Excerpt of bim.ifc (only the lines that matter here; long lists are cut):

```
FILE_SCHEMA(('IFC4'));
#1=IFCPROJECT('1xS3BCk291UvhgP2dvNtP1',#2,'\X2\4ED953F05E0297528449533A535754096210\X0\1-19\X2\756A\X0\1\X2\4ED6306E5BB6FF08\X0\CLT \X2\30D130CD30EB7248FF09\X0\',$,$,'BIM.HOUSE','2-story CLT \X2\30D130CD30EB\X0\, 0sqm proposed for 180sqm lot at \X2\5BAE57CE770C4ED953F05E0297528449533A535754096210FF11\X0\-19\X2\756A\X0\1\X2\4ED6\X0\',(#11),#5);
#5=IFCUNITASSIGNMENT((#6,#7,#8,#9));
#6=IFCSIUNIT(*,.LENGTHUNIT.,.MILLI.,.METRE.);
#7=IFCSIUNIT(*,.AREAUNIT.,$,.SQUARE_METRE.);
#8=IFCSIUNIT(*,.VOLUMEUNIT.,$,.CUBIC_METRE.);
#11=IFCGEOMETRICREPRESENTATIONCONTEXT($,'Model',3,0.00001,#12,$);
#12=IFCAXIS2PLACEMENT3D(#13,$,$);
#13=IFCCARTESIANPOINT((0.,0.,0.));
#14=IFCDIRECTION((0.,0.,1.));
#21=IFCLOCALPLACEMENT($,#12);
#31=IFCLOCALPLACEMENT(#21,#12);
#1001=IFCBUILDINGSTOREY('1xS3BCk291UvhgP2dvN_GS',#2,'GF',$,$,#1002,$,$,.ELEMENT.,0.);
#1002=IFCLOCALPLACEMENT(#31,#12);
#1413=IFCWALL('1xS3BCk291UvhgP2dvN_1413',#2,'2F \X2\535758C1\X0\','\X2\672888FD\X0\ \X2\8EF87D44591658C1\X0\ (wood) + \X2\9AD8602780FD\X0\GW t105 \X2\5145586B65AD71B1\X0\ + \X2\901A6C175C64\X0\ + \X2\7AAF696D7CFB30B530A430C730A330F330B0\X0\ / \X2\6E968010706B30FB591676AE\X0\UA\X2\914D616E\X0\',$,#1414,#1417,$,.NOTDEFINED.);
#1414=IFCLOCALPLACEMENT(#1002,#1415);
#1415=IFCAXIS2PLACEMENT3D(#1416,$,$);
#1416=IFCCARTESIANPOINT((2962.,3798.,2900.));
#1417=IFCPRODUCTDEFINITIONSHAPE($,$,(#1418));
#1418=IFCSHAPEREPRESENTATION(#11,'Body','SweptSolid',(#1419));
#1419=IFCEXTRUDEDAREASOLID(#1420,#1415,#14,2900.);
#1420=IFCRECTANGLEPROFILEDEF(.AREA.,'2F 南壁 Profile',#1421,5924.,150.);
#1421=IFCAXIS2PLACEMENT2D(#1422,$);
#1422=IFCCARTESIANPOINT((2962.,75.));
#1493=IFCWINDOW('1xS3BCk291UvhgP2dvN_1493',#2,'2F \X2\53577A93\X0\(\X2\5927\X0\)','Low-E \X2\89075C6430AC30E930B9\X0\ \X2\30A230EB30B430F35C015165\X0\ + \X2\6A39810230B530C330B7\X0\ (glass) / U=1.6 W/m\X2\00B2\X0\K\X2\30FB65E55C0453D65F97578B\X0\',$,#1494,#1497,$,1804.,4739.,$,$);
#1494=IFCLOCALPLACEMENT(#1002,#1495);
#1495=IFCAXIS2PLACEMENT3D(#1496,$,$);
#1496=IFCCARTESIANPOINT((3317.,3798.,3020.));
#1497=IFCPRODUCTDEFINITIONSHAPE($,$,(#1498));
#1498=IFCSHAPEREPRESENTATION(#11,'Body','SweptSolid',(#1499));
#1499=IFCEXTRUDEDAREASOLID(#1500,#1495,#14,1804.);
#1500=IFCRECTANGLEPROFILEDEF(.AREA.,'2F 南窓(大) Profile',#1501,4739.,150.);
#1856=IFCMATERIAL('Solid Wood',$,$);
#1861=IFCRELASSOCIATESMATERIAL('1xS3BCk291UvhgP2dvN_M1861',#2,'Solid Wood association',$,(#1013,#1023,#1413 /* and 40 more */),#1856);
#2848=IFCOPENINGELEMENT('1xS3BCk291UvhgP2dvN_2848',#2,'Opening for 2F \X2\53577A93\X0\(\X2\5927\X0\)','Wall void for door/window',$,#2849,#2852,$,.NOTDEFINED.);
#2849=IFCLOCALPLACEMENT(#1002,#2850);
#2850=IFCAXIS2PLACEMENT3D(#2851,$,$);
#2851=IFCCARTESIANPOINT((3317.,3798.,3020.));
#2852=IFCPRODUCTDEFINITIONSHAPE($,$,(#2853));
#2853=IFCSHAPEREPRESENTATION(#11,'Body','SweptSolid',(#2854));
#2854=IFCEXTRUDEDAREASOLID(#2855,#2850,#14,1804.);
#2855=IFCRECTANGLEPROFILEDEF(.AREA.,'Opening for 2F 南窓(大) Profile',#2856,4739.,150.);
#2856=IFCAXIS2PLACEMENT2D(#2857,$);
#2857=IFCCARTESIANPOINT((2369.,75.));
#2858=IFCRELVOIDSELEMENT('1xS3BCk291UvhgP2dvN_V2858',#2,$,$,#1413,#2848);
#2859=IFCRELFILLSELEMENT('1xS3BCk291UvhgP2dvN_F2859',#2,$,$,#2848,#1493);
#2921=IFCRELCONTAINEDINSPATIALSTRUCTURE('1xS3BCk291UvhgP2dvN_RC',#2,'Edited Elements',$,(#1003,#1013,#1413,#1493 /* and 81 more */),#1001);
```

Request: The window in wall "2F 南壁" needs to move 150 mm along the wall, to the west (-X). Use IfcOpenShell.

```python
import ifcopenshell
import ifcopenshell.api.geometry
import ifcopenshell.util.placement
import ifcopenshell.util.unit

model = ifcopenshell.open("bim.ifc")
unit_scale = ifcopenshell.util.unit.calculate_unit_scale(model)

window = model.by_id(1493)
opening = window.FillsVoids[0].RelatingOpeningElement
wall = opening.VoidsElements[0].RelatingBuildingElement

wall_matrix = ifcopenshell.util.placement.get_local_placement(wall.ObjectPlacement)
shift = wall_matrix[:3, 0] * -0.15 / unit_scale
before = ifcopenshell.util.placement.get_local_placement(window.ObjectPlacement)[:3, 3].copy()

# The window is not placed relative to its opening, so move both.
for product in (opening, window):
    matrix = ifcopenshell.util.placement.get_local_placement(product.ObjectPlacement)
    matrix[:3, 3] += shift
    ifcopenshell.api.geometry.edit_object_placement(model, product=product, matrix=matrix, is_si=False)

after = ifcopenshell.util.placement.get_local_placement(window.ObjectPlacement)[:3, 3]
print("window moved by", (after - before).round(3) + 0.0)

model.write("bim_rev.ifc")
```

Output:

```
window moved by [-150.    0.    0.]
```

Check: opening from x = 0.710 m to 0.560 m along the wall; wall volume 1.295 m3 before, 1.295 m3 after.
